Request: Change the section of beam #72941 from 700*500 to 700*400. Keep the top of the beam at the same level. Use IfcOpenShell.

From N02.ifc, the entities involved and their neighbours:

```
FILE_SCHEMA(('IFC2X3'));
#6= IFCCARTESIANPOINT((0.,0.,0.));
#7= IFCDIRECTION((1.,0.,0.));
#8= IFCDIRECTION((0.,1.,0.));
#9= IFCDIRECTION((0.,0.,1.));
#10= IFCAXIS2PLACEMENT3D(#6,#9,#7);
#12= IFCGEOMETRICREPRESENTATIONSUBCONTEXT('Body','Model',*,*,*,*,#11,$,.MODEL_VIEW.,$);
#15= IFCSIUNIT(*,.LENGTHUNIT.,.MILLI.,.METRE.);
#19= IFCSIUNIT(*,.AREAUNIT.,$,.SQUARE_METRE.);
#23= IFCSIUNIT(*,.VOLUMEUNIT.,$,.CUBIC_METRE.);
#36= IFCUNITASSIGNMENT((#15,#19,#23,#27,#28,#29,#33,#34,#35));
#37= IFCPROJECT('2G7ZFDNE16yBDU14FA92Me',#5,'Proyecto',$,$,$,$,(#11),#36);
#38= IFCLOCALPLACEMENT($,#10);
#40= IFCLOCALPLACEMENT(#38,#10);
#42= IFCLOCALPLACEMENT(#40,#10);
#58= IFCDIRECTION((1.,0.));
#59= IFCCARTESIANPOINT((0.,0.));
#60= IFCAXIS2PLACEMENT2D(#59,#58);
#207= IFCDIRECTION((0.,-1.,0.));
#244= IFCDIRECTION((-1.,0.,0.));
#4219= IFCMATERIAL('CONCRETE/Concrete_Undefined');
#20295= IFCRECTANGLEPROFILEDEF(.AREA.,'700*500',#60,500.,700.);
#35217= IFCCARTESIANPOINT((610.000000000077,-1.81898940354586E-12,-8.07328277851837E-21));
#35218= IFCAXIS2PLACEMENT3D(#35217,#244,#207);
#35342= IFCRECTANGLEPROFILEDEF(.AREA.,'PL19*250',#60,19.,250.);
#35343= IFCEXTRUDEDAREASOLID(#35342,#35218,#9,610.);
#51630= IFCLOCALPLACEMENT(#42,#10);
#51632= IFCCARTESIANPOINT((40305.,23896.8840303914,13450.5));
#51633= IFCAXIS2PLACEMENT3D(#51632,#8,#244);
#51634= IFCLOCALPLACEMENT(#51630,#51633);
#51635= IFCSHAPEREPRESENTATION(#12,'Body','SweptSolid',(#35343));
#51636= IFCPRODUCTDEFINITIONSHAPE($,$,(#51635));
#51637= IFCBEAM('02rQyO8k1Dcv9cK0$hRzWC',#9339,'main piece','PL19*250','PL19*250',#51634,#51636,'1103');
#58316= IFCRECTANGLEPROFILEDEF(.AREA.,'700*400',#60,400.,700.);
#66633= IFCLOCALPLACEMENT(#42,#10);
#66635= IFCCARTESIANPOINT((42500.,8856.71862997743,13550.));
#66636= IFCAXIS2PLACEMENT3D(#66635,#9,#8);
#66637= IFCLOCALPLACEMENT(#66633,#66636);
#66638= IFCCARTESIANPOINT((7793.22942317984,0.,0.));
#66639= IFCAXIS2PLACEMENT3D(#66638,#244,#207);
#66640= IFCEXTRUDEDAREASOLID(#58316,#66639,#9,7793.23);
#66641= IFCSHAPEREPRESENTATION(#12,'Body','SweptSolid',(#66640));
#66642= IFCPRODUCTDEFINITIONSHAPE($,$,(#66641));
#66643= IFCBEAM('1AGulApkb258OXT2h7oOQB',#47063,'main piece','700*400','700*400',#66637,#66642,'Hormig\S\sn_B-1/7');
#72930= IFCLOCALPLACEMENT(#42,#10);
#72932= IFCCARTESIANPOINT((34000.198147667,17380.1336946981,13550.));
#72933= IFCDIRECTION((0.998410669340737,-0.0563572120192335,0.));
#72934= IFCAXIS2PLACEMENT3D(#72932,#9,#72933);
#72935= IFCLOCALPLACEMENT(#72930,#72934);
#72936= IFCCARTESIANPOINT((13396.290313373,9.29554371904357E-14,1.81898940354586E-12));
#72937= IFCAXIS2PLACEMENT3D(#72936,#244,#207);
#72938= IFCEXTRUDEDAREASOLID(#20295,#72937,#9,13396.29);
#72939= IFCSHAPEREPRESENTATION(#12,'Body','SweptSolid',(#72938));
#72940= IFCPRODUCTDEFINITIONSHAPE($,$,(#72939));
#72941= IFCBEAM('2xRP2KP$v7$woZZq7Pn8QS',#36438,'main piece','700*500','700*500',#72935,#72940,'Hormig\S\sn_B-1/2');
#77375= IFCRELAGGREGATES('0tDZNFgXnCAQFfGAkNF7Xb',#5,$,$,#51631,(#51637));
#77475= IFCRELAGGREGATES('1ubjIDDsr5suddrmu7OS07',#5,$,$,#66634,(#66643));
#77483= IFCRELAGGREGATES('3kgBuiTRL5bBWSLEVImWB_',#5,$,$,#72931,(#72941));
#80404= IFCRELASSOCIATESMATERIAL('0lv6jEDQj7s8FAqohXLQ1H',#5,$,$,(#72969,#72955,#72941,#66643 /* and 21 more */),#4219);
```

```python
import ifcopenshell
import ifcopenshell.util.element
import ifcopenshell.util.representation

model = ifcopenshell.open("N02.ifc")

member = model.by_guid("2xRP2KP$v7$woZZq7Pn8QS")
source = next(p for p in model.by_type("IfcRectangleProfileDef") if p.ProfileName == "700*400")

body = ifcopenshell.util.representation.get_representation(member, "Model", "Body")
solid = body.Items[0]
old_profile = solid.SweptArea

# Copy the section's sizes but keep this member's own profile position.
profile = ifcopenshell.util.element.copy(model, source)
# Profiles are centred, so shift by half the change in depth to hold the top.
shift = (old_profile.YDim - profile.YDim) / 2
x, y = old_profile.Position.Location.Coordinates
up = (0.0, 1.0)  # upwards, in the solid's own plane
location = model.createIfcCartesianPoint((x + up[0] * shift, y + up[1] * shift))
profile.Position = model.createIfcAxis2Placement2D(location, old_profile.Position.RefDirection)
solid.SweptArea = profile
if not model.get_total_inverses(old_profile):
    ifcopenshell.util.element.remove_deep2(model, old_profile)
member.Description = member.Description.replace("700*500", "700*400")
member.ObjectType = member.ObjectType.replace("700*500", "700*400")

print(solid.SweptArea)

model.write("N02_updated.ifc")
```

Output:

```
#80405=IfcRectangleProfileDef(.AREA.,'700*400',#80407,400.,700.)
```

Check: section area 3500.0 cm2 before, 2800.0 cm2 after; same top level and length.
